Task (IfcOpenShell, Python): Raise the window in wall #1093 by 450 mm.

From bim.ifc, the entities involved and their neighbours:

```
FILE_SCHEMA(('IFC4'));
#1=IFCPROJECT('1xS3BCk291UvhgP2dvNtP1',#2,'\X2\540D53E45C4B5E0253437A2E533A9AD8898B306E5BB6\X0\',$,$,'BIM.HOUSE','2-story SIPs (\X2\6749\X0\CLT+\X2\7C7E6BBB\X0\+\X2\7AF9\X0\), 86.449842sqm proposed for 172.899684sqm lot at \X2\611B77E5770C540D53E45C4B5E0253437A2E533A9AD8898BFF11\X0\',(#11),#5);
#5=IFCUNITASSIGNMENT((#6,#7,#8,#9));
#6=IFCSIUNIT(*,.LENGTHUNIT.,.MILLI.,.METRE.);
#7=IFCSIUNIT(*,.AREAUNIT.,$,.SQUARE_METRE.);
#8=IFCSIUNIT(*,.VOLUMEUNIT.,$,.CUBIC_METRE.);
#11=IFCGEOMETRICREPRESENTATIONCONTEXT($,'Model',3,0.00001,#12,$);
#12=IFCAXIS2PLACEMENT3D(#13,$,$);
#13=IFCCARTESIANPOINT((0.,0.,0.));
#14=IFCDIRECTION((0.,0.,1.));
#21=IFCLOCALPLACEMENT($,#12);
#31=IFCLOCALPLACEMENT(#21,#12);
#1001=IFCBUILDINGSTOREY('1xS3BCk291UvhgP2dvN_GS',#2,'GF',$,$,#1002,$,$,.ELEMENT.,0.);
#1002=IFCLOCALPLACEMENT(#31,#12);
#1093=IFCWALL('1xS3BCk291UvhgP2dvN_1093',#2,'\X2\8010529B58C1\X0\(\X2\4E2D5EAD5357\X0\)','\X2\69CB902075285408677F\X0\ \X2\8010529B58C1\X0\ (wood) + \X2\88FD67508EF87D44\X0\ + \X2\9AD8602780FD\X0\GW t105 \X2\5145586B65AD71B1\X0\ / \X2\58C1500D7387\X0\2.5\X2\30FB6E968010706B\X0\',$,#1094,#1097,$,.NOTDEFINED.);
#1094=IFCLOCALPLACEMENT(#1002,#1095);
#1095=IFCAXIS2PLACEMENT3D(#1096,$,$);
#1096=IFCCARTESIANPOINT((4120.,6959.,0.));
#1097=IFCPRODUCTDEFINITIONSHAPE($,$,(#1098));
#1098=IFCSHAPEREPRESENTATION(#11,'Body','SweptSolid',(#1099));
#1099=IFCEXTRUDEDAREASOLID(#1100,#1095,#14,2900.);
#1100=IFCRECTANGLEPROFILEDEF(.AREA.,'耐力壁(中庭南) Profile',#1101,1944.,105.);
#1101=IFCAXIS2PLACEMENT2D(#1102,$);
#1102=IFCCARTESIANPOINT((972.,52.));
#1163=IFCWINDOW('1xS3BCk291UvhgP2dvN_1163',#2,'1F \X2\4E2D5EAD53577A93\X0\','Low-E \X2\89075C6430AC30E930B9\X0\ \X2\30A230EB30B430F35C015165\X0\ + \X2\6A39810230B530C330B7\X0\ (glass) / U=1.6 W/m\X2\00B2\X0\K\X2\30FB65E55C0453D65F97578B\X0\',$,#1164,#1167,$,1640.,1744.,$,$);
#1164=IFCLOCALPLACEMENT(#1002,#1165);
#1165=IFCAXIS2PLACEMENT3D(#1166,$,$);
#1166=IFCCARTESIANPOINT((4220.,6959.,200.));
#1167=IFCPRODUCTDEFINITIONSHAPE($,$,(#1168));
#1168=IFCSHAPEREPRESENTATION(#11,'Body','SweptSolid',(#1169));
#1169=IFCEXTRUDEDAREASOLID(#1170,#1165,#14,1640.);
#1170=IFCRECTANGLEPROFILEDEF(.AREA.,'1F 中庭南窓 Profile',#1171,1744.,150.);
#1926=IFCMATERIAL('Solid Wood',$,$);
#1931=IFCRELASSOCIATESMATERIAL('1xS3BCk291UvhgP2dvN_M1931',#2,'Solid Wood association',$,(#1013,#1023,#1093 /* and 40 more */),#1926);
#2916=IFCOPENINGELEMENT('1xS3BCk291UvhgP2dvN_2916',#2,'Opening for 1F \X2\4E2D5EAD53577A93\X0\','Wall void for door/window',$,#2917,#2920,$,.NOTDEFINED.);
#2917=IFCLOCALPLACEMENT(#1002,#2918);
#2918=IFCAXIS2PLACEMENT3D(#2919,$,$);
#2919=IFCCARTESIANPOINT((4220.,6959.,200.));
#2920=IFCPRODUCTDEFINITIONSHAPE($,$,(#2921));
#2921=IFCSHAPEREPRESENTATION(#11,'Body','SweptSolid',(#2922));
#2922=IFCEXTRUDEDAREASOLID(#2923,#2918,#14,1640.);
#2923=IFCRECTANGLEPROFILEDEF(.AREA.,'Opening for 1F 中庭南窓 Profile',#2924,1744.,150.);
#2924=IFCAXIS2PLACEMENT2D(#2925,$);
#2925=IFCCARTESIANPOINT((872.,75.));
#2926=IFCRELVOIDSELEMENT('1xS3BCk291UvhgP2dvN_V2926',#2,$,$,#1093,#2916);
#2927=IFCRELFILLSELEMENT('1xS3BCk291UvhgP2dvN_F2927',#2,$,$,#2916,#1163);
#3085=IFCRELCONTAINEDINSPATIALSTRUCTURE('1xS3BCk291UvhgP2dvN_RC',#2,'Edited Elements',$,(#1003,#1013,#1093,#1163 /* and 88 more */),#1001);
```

```python
import numpy as np
import ifcopenshell
import ifcopenshell.api.geometry
import ifcopenshell.util.placement
import ifcopenshell.util.unit

model = ifcopenshell.open("bim.ifc")
unit_scale = ifcopenshell.util.unit.calculate_unit_scale(model)

window = model.by_guid("1xS3BCk291UvhgP2dvN_1163")
opening = window.FillsVoids[0].RelatingOpeningElement
dz = 450.0

shift = np.array([0.0, 0.0, dz])
# The window is not placed relative to its opening, so move both.
for product in (opening, window):
    matrix = ifcopenshell.util.placement.get_local_placement(product.ObjectPlacement)
    matrix[:3, 3] += shift
    ifcopenshell.api.geometry.edit_object_placement(model, product=product, matrix=matrix, is_si=False)

print(f"moved by {dz * unit_scale:+.3f} m")

model.write("bim_rev.ifc")
```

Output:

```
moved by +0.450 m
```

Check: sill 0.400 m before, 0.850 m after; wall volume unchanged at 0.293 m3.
